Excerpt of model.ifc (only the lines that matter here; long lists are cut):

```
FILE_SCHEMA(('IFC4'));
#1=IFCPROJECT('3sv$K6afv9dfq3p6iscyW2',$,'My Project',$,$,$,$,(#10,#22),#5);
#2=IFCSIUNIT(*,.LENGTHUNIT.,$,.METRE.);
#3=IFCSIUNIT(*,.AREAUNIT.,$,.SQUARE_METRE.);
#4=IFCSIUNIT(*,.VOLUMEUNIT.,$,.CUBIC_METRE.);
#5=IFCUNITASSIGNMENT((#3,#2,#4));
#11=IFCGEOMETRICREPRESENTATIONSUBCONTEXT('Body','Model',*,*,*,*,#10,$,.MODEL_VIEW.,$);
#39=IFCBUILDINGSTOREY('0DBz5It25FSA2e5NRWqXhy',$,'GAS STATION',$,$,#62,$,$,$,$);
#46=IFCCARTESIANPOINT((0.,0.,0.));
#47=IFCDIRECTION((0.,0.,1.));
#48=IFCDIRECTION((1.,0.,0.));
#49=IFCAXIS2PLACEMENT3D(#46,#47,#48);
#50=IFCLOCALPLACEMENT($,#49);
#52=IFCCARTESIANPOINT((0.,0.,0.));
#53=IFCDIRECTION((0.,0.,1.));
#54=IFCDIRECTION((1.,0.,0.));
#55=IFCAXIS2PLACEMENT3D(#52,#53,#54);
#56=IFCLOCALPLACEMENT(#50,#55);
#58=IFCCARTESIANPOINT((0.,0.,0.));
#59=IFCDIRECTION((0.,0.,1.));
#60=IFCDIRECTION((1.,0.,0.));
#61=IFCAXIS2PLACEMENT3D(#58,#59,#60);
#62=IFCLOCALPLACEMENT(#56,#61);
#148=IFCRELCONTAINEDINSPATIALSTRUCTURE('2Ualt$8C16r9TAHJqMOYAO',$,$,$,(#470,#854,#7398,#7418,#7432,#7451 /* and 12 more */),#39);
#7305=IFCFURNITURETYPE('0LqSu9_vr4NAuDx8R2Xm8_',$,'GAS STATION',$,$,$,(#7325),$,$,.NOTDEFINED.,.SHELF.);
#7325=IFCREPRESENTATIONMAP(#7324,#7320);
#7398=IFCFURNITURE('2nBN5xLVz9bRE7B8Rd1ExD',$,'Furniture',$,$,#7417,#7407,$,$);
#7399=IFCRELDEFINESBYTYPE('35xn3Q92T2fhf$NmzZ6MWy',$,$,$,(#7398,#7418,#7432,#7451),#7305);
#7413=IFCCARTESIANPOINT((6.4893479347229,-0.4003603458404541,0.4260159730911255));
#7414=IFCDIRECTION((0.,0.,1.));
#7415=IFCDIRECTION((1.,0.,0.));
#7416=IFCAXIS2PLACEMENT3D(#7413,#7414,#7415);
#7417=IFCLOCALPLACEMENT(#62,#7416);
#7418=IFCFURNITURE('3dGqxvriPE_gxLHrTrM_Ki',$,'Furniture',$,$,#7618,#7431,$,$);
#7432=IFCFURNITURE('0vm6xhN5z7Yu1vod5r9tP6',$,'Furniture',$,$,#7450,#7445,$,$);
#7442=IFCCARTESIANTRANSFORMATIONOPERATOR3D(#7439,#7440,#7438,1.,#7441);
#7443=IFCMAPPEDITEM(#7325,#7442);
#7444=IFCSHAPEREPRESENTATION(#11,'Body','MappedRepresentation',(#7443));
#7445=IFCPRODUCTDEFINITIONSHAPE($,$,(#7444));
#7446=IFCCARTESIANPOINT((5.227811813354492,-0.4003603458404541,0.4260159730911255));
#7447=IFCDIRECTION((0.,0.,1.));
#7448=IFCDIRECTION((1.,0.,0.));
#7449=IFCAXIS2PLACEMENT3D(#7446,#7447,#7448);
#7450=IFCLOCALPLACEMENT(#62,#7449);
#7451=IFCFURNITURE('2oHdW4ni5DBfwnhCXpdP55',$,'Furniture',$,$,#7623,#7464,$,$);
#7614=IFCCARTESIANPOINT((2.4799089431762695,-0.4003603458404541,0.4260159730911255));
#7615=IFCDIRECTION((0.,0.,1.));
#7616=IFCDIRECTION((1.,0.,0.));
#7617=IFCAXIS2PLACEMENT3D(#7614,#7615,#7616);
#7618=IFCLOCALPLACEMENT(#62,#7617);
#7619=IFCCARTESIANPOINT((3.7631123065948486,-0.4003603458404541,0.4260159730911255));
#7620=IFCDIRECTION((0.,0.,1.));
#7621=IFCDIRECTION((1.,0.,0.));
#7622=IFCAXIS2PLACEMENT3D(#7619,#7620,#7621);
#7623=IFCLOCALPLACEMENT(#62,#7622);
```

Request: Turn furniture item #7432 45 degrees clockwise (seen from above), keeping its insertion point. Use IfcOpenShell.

```python
import ifcopenshell
import ifcopenshell.api.geometry
import ifcopenshell.util.placement

model = ifcopenshell.open("model.ifc")

item = model.by_guid("0vm6xhN5z7Yu1vod5r9tP6")
matrix = ifcopenshell.util.placement.get_local_placement(item.ObjectPlacement)
matrix = matrix @ ifcopenshell.util.placement.rotation(-45, "Z")
ifcopenshell.api.geometry.edit_object_placement(model, product=item, matrix=matrix, is_si=False)

print(ifcopenshell.util.placement.get_local_placement(item.ObjectPlacement).round(3) + 0.0)

model.write("model_updated.ifc")
```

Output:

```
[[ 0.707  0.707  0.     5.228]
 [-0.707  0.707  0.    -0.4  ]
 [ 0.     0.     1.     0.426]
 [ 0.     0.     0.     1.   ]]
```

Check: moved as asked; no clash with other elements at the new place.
